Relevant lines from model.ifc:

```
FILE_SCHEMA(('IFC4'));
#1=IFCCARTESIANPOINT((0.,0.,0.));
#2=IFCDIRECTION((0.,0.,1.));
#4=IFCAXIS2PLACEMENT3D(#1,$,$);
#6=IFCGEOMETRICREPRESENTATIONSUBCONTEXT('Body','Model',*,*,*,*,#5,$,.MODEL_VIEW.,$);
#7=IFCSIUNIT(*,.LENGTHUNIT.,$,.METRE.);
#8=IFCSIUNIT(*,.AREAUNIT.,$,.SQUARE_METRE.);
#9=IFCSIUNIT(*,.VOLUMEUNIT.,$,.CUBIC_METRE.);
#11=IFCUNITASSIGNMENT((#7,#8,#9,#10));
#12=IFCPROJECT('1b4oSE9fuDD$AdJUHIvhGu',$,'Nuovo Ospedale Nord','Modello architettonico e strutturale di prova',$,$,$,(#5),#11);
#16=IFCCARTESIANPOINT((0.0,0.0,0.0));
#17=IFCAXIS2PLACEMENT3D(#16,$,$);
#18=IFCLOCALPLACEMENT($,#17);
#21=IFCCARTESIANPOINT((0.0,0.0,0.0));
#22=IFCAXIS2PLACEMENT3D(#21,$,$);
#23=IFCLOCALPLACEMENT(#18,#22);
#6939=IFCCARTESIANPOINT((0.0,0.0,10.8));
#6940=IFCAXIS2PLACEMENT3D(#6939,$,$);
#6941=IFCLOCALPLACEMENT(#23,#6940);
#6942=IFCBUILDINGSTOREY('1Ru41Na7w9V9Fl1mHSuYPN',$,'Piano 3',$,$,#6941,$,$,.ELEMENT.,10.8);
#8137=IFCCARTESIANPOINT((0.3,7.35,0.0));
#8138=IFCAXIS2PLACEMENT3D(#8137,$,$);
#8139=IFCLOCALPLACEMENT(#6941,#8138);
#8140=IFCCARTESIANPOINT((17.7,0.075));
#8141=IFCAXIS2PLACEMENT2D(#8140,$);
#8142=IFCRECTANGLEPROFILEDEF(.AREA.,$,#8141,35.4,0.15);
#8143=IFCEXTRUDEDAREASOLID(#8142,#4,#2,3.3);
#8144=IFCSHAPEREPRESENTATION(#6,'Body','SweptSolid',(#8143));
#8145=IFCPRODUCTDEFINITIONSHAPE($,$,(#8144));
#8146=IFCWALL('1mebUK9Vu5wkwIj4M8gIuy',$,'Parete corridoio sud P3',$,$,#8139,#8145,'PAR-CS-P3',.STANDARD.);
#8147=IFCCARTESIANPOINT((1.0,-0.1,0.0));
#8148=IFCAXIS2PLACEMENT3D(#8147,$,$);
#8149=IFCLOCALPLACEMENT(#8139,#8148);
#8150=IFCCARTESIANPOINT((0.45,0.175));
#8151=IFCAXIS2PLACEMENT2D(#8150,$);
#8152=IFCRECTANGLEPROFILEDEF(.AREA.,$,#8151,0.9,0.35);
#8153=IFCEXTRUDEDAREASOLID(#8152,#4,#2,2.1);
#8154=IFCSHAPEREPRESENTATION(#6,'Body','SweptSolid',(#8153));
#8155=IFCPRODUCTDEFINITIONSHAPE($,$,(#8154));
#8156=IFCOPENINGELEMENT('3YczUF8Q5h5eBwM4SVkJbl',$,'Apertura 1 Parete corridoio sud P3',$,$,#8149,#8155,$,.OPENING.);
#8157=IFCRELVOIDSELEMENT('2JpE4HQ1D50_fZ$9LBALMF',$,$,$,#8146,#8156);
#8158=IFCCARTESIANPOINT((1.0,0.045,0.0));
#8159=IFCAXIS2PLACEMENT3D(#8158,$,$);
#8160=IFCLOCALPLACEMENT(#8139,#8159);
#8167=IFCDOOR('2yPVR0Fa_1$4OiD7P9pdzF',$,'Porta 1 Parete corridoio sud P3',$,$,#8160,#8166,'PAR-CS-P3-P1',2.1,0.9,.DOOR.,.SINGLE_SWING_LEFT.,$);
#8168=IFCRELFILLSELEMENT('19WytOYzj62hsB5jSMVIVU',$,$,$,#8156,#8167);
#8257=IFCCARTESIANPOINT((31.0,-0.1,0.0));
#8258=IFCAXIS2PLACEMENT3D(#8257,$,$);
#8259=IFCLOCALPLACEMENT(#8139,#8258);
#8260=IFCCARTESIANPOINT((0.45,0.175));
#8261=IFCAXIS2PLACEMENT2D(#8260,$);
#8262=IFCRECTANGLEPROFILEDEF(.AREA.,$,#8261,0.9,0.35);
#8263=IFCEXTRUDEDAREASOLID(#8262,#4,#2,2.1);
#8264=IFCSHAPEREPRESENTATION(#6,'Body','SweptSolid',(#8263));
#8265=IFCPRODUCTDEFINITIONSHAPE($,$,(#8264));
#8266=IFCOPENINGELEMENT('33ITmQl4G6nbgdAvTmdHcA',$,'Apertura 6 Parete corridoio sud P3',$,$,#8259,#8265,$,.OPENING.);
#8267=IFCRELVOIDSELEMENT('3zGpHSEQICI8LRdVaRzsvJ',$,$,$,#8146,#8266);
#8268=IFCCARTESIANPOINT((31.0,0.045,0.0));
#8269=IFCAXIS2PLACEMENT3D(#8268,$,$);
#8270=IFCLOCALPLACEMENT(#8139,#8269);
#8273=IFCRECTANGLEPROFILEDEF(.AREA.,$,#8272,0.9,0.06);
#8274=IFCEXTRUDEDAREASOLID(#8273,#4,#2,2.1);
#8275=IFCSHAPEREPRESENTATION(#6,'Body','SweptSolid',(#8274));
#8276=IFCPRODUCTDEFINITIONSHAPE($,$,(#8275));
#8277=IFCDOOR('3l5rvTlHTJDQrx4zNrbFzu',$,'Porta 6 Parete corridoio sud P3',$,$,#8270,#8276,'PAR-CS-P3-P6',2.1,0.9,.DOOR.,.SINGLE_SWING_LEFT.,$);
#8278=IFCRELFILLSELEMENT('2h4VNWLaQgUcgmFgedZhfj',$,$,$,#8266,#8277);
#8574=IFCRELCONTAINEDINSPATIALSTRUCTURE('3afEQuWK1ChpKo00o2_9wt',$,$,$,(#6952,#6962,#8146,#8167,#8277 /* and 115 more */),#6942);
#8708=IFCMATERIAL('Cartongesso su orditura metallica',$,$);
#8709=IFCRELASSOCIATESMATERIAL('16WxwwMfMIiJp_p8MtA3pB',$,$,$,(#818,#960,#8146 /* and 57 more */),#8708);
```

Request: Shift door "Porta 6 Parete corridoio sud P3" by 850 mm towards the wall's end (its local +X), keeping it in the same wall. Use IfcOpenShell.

```python
import ifcopenshell
import ifcopenshell.api.geometry
import ifcopenshell.util.placement

model = ifcopenshell.open("model.ifc")

door = model.by_guid("3l5rvTlHTJDQrx4zNrbFzu")
opening = door.FillsVoids[0].RelatingOpeningElement
wall = opening.VoidsElements[0].RelatingBuildingElement

wall_matrix = ifcopenshell.util.placement.get_local_placement(wall.ObjectPlacement)
shift = wall_matrix[:3, 0] * 0.85
before = ifcopenshell.util.placement.get_local_placement(door.ObjectPlacement)[:3, 3].copy()

# The door is not placed relative to its opening, so move both.
for product in (opening, door):
    matrix = ifcopenshell.util.placement.get_local_placement(product.ObjectPlacement)
    matrix[:3, 3] += shift
    ifcopenshell.api.geometry.edit_object_placement(model, product=product, matrix=matrix, is_si=False)

after = ifcopenshell.util.placement.get_local_placement(door.ObjectPlacement)[:3, 3]
print("door moved by", (after - before).round(3) + 0.0)

model.write("model_updated.ifc")
```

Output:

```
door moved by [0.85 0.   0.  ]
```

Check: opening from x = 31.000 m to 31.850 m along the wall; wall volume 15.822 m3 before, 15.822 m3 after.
